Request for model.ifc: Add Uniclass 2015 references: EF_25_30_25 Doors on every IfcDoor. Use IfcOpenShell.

First a look at what the model holds.

```python
import ifcopenshell

model = ifcopenshell.open("model.ifc")
print(model.schema)
print("classifications:", [c.Name for c in model.by_type("IfcClassification")])
for ifc_class in ("IfcDoor", "IfcRoof", "IfcStair", "IfcWall", "IfcWindow"):
    print(ifc_class, len(model.by_type(ifc_class)))
```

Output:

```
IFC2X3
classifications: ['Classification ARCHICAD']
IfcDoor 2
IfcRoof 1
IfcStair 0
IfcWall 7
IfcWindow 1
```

```python
import ifcopenshell
import ifcopenshell.api.classification

model = ifcopenshell.open("model.ifc")

# IFC2X3 requires Source and Edition and has no link from the project to the system.
system = model.create_entity("IfcClassification", Source="NBS", Edition="2015", Name="Uniclass 2015")

codes = {
    "IfcDoor": ("EF_25_30_25", "Doors"),
}
for ifc_class, (code, name) in codes.items():
    products = model.by_type(ifc_class)
    ifcopenshell.api.classification.add_reference(
        model, products=products, classification=system, identification=code, name=name
    )
    print(code, len(products))

model.write("model_updated.ifc")
```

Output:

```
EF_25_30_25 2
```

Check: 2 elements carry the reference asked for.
